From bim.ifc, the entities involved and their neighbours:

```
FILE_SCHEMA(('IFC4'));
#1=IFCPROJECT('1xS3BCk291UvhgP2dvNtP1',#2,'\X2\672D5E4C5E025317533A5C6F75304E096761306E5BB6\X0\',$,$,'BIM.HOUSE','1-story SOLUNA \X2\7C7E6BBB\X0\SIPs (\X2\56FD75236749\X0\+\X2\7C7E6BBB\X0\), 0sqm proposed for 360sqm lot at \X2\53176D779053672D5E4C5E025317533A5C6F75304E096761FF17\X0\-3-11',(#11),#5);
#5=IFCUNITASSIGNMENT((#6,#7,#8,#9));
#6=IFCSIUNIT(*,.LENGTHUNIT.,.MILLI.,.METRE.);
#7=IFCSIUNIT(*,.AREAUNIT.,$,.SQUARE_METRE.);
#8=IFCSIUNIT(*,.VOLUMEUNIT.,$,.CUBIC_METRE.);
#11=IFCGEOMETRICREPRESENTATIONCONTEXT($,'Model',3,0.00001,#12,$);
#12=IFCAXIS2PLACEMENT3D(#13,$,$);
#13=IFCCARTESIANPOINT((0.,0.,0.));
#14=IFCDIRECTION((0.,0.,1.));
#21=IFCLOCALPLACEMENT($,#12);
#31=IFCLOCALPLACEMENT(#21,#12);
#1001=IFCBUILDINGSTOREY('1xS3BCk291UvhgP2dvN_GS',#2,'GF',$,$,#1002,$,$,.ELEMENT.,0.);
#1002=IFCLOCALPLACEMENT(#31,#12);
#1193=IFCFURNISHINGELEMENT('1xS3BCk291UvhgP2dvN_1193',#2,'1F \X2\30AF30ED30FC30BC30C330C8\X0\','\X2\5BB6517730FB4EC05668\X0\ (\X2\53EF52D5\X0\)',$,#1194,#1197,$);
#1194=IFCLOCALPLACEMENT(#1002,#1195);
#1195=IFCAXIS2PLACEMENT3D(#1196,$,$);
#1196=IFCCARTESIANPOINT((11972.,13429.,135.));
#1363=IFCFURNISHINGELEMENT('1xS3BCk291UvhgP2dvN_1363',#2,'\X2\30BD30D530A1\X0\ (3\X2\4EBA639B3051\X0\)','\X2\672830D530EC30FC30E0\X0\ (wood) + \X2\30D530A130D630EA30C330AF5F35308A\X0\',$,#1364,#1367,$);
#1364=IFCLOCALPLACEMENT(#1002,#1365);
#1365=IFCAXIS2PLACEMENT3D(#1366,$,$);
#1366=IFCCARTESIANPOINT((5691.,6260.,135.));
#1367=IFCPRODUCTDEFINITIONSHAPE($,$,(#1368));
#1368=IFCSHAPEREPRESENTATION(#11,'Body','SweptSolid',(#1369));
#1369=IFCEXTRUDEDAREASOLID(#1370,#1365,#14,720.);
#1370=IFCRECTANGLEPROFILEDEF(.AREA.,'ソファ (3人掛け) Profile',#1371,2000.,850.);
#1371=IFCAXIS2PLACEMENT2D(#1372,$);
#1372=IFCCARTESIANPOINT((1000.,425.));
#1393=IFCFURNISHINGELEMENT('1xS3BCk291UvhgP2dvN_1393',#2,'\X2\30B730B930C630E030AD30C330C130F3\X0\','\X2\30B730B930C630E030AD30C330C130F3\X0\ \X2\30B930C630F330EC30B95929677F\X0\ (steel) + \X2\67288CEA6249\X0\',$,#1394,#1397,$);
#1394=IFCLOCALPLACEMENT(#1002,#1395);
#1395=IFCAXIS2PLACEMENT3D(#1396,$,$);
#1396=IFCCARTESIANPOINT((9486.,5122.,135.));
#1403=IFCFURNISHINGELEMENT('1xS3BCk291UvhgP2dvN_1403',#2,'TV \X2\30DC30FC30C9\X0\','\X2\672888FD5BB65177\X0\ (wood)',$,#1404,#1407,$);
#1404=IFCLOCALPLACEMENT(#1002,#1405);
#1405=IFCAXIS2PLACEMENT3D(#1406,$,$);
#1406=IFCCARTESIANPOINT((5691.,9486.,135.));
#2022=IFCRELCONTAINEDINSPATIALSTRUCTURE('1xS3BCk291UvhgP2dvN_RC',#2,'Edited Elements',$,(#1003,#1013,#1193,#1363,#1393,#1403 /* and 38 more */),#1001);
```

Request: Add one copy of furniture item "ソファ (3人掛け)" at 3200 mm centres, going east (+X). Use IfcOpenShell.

```python
import numpy as np
import ifcopenshell
import ifcopenshell.api.geometry
import ifcopenshell.api.root
import ifcopenshell.util.element
import ifcopenshell.util.placement
import ifcopenshell.util.unit

model = ifcopenshell.open("bim.ifc")
unit_scale = ifcopenshell.util.unit.calculate_unit_scale(model)


def reuse_history(source, copy):
    """copy_class also copies each property set's owner history, people and application; keep the originals."""
    for rel in copy.IsDefinedBy:
        if rel.is_a("IfcRelDefinesByProperties") and (history := rel.RelatingPropertyDefinition.OwnerHistory):
            rel.RelatingPropertyDefinition.OwnerHistory = source.OwnerHistory
            ifcopenshell.util.element.remove_deep2(model, history)


source = model.by_guid("1xS3BCk291UvhgP2dvN_1363")
base = ifcopenshell.util.placement.get_local_placement(source.ObjectPlacement)
step = np.array([1.0, 0.0, 0.0]) * 3.2 / unit_scale

for i in range(1, 2):
    copy = ifcopenshell.api.root.copy_class(model, product=source)
    copy.Representation = ifcopenshell.util.element.copy_deep(
        model, source.Representation, exclude=["IfcGeometricRepresentationContext", "IfcRepresentationMap"]
    )
    reuse_history(source, copy)
    matrix = base.copy()
    matrix[:3, 3] += i * step
    print("added at", matrix[:3, 3].round(3) + 0.0)
    ifcopenshell.api.geometry.edit_object_placement(model, product=copy, matrix=matrix, is_si=False)

model.write("bim_edited.ifc")
```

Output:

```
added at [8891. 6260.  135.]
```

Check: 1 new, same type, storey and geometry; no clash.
